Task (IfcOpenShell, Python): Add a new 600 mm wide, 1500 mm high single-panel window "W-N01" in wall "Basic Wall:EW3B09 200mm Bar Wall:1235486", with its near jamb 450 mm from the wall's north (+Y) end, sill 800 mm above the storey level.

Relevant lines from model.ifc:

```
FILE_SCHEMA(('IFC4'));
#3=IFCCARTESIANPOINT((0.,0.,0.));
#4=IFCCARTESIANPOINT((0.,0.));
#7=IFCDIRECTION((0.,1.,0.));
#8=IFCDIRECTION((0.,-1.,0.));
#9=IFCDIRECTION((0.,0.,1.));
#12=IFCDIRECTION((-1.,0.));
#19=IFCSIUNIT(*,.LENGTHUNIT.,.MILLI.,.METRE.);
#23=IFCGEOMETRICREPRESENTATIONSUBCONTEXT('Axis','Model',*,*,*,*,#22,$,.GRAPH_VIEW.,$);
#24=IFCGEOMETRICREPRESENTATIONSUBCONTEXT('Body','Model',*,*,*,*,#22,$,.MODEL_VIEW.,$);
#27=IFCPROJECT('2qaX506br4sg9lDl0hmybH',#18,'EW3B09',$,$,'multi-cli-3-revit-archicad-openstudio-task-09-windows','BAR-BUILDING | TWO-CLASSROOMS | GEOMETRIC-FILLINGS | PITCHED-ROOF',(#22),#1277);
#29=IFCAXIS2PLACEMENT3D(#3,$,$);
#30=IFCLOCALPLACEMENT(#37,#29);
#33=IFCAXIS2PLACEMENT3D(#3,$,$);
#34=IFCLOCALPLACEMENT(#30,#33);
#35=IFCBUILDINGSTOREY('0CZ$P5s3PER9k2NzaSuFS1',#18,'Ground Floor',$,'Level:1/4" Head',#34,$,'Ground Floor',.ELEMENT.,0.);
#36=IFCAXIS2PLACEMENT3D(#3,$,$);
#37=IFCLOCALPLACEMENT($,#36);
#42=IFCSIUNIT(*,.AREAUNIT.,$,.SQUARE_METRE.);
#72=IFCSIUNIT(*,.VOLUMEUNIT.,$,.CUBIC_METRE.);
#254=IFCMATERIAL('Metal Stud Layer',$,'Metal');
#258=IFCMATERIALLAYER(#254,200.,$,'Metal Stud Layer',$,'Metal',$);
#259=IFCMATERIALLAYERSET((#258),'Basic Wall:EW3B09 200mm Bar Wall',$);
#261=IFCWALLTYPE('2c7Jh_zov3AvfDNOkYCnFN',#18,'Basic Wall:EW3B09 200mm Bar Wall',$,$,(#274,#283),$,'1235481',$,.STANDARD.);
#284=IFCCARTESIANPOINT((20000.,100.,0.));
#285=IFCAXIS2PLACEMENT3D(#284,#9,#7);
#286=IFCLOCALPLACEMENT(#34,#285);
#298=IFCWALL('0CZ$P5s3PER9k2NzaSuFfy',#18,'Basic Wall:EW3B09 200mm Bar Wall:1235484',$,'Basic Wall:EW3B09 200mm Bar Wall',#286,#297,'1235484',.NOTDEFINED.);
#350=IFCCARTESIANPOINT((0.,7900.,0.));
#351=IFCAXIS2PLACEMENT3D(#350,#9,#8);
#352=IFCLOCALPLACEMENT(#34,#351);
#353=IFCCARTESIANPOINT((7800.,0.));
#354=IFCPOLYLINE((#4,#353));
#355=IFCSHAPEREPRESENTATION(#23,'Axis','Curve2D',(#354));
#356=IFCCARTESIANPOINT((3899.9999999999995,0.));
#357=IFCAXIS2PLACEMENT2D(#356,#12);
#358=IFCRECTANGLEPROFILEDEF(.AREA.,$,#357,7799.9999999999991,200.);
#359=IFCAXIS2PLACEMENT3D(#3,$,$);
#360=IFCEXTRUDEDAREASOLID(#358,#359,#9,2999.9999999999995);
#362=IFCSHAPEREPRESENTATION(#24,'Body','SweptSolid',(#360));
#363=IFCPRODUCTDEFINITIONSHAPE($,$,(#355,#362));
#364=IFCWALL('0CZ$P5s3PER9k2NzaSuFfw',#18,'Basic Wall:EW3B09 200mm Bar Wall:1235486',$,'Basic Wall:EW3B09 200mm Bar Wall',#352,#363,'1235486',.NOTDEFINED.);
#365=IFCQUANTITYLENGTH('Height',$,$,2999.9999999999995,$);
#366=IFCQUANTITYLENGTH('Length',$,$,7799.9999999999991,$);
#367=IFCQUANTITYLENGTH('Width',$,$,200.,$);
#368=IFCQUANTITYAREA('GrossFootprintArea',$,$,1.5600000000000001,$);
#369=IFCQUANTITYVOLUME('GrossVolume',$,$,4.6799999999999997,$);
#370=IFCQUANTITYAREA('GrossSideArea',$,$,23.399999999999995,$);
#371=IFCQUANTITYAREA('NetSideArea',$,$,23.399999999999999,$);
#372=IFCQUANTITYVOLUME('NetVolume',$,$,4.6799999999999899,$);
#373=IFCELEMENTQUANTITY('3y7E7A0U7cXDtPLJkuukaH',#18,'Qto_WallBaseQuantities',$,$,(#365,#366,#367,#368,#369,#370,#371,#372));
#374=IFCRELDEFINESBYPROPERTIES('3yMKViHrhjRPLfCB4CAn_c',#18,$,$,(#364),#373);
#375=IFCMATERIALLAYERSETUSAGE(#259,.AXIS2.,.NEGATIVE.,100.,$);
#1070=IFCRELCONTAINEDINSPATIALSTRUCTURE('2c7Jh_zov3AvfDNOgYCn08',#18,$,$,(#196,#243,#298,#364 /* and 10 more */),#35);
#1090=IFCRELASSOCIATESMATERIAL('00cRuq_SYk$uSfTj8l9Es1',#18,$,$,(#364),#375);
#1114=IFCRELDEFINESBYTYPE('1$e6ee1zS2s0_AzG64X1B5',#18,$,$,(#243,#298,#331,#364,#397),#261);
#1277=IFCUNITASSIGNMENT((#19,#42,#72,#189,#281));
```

```python
import numpy as np
import ifcopenshell
import ifcopenshell.api.feature
import ifcopenshell.api.geometry
import ifcopenshell.api.pset
import ifcopenshell.api.root
import ifcopenshell.api.spatial
import ifcopenshell.geom
import ifcopenshell.util.element
import ifcopenshell.util.placement
import ifcopenshell.util.representation
import ifcopenshell.util.shape
import ifcopenshell.util.unit

model = ifcopenshell.open("model.ifc")
unit_scale = ifcopenshell.util.unit.calculate_unit_scale(model)
area_scale = ifcopenshell.util.unit.calculate_unit_scale(model, "AREAUNIT")
volume_scale = ifcopenshell.util.unit.calculate_unit_scale(model, "VOLUMEUNIT")
settings = ifcopenshell.geom.settings()


def volume(element):
    """Net volume in cubic metres, openings subtracted."""
    shape = ifcopenshell.geom.create_shape(settings, element)
    return ifcopenshell.util.shape.get_volume(shape.geometry)


wall = model.by_id(364)
storey = ifcopenshell.util.element.get_container(wall, ifc_class="IfcBuildingStorey")
context = ifcopenshell.util.representation.get_context(model, "Model", "Body", "MODEL_VIEW")
before = volume(wall)

width, height, from_end, sill = 0.6, 1.5, 0.45, 0.8  # metres

# The wall runs along its own X axis, and the end named is its -X end.
wall_shape = ifcopenshell.geom.create_shape(settings, wall)
x, y, z = ifcopenshell.util.shape.get_vertices(wall_shape.geometry).T
start = x.min() + from_end
face, thickness = float(y.min()), float(y.max() - y.min())
wall_matrix = ifcopenshell.util.placement.get_local_placement(wall.ObjectPlacement)
level = ifcopenshell.util.placement.get_local_placement(storey.ObjectPlacement)[2, 3]


def in_wall(x, y):
    """Placement at x, y metres in the wall's axes, at sill height."""
    matrix = wall_matrix.copy()
    matrix[:, 3] = wall_matrix @ np.array([x / unit_scale, y / unit_scale, 0.0, 1.0])
    matrix[2, 3] = level + sill / unit_scale
    return matrix


# Opening: a box that overshoots both wall faces by 50 mm.
opening = ifcopenshell.api.root.create_entity(model, ifc_class="IfcOpeningElement", predefined_type="OPENING")
box = ifcopenshell.api.geometry.add_wall_representation(
    model, context=context, length=width, height=height, thickness=thickness + 0.1
)
ifcopenshell.api.geometry.assign_representation(model, product=opening, representation=box)
ifcopenshell.api.geometry.edit_object_placement(model, product=opening, matrix=in_wall(start, face - 0.05), is_si=False)
ifcopenshell.api.feature.add_feature(model, feature=opening, element=wall)

window = ifcopenshell.api.root.create_entity(model, ifc_class="IfcWindow", name="W-N01", predefined_type="WINDOW")
window.OverallWidth, window.OverallHeight = width / unit_scale, height / unit_scale
window.PartitioningType = "SINGLE_PANEL"
body = ifcopenshell.api.geometry.add_window_representation(
    model,
    context=context,
    overall_width=window.OverallWidth,
    overall_height=window.OverallHeight,
    partition_type="SINGLE_PANEL",
)
ifcopenshell.api.geometry.assign_representation(model, product=window, representation=body)
ifcopenshell.api.spatial.assign_container(model, products=[window], relating_structure=storey)
ifcopenshell.api.feature.add_filling(model, opening=opening, element=window)

# Centre the window in the wall's thickness.
ifcopenshell.api.geometry.edit_object_placement(model, product=window, matrix=in_wall(start, face), is_si=False)
window_shape = ifcopenshell.geom.create_shape(settings, window)
depth = ifcopenshell.util.shape.get_vertices(window_shape.geometry)[:, 1]
offset = face + thickness / 2 - (depth.min() + depth.max()) / 2
ifcopenshell.api.geometry.edit_object_placement(model, product=window, matrix=in_wall(start, offset), is_si=False)

after = volume(wall)

# Update the wall's stored quantities.
qto = model.by_id(ifcopenshell.util.element.get_pset(wall, "Qto_WallBaseQuantities", should_inherit=False)["id"])
ifcopenshell.api.pset.edit_qto(model, qto=qto, properties={
    "NetSideArea": after / thickness / area_scale,
    "NetVolume": after / volume_scale,
})

print(f"wall volume {before:.3f} -> {after:.3f} m3")

model.write("model_v2.ifc")
```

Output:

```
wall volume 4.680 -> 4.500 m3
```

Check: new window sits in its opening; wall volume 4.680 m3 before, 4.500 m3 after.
